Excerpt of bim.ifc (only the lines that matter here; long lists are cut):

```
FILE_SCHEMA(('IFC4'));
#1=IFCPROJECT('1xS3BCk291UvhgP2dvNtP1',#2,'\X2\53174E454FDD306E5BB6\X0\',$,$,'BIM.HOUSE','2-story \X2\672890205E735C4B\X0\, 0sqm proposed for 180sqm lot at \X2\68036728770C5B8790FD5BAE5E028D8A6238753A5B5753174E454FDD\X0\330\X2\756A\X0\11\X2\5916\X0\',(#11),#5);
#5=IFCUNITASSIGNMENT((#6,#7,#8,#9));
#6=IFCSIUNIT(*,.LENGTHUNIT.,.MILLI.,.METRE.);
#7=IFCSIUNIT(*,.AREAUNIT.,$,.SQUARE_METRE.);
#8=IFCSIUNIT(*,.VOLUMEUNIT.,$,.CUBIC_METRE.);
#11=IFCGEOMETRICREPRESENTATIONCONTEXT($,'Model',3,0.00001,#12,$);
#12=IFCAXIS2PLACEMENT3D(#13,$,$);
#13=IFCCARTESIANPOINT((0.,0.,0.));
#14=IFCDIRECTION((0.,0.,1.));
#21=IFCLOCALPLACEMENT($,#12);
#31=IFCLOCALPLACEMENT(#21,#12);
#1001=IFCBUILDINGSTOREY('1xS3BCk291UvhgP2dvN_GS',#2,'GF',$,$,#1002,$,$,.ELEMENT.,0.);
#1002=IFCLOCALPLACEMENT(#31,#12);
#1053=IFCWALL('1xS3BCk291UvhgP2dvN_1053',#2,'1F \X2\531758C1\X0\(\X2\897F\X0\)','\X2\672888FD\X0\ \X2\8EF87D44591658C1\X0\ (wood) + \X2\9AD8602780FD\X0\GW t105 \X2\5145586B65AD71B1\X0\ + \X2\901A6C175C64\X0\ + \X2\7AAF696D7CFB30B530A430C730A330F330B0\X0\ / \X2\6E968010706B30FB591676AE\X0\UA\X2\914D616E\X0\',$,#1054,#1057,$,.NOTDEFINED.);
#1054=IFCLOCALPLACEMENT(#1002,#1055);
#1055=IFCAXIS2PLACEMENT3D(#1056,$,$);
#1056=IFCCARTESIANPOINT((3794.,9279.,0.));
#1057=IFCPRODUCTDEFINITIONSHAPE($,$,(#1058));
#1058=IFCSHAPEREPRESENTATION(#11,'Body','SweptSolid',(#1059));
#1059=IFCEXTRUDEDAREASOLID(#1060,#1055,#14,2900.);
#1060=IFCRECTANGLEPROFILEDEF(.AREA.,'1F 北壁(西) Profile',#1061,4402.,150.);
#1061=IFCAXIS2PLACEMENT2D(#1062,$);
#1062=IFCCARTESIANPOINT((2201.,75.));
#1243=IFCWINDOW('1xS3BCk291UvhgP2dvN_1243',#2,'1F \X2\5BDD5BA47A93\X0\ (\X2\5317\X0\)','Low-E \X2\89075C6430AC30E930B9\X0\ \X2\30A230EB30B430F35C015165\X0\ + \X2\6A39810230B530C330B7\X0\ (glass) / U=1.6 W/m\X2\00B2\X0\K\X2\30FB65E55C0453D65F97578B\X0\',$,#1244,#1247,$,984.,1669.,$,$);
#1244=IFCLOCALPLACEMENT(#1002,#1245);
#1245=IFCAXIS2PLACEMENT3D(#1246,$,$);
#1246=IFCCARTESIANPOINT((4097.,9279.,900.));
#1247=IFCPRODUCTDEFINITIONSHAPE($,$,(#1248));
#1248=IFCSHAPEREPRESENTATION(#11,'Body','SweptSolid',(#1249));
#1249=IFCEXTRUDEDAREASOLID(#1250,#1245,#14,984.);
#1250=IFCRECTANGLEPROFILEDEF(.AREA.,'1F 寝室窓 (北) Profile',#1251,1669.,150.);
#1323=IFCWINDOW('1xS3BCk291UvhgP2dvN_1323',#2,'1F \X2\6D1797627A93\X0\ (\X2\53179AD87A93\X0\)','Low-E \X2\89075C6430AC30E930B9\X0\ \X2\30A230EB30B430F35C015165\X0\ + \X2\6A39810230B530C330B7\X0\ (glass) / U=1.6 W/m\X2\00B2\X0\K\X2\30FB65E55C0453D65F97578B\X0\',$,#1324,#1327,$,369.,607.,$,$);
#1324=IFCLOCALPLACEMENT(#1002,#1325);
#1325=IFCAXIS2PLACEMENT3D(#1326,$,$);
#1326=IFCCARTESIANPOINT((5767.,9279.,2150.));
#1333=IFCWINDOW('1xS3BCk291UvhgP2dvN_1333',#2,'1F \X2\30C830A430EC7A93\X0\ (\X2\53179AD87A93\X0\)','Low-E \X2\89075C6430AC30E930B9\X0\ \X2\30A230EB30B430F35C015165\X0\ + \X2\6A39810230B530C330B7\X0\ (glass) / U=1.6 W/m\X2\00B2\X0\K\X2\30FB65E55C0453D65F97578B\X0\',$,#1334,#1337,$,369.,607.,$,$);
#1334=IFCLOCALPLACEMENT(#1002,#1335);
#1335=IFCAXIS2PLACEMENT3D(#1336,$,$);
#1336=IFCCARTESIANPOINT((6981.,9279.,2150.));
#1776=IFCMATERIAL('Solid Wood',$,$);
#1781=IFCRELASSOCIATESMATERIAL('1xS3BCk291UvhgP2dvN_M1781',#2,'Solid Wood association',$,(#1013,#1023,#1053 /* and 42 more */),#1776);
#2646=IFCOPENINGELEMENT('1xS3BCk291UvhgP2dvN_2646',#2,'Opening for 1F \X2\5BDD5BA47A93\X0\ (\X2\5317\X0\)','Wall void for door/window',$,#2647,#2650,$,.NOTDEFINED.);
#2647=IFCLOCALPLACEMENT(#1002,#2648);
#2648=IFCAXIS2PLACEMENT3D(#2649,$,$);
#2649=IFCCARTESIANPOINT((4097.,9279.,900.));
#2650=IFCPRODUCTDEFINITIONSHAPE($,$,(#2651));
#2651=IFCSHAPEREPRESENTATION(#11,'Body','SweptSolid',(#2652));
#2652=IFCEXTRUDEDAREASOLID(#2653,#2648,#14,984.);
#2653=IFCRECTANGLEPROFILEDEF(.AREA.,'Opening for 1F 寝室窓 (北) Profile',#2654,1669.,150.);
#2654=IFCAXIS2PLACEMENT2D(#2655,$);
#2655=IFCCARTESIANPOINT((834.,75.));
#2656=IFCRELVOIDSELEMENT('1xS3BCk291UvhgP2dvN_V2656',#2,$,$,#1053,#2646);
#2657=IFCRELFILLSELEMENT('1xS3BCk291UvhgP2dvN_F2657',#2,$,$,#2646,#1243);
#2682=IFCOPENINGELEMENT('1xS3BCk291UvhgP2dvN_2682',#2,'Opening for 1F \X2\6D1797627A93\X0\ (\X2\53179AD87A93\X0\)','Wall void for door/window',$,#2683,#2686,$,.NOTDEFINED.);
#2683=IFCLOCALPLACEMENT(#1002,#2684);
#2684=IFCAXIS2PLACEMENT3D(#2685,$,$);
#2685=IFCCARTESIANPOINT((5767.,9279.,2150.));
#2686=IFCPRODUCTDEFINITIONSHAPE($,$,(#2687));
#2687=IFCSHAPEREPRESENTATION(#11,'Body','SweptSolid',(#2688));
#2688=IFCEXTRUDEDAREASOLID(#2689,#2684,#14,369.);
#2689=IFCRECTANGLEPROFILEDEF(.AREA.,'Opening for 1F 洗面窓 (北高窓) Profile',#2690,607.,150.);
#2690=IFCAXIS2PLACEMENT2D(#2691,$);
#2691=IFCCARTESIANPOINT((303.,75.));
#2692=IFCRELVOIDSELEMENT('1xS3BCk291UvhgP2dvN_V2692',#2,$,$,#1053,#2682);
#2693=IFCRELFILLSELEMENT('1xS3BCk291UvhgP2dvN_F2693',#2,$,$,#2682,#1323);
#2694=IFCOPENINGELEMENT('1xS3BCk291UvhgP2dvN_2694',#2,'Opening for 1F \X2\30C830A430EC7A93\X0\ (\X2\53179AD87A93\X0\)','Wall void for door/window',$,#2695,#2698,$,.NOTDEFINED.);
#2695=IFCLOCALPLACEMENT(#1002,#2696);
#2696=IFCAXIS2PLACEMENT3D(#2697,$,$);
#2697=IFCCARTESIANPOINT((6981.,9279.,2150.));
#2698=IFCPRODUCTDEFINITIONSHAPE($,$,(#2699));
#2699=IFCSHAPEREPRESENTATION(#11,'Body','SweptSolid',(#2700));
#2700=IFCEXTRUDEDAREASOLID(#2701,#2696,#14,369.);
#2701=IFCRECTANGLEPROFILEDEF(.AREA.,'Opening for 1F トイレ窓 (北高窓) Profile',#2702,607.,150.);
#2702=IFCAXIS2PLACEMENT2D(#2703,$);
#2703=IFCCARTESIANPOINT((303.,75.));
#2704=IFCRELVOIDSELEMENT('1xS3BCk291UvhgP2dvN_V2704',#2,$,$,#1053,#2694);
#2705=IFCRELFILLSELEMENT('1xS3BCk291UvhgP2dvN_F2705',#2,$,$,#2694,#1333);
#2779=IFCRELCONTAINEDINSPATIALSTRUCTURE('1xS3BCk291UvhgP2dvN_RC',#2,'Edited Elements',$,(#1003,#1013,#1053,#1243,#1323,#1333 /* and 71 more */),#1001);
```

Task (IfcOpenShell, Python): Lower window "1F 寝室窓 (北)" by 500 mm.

```python
import numpy as np
import ifcopenshell
import ifcopenshell.api.geometry
import ifcopenshell.util.placement
import ifcopenshell.util.unit

model = ifcopenshell.open("bim.ifc")
unit_scale = ifcopenshell.util.unit.calculate_unit_scale(model)

window = model.by_guid("1xS3BCk291UvhgP2dvN_1243")
opening = window.FillsVoids[0].RelatingOpeningElement
dz = -500.0

shift = np.array([0.0, 0.0, dz])
# The window is not placed relative to its opening, so move both.
for product in (opening, window):
    matrix = ifcopenshell.util.placement.get_local_placement(product.ObjectPlacement)
    matrix[:3, 3] += shift
    ifcopenshell.api.geometry.edit_object_placement(model, product=product, matrix=matrix, is_si=False)

print(f"moved by {dz * unit_scale:+.3f} m")

model.write("bim-out.ifc")
```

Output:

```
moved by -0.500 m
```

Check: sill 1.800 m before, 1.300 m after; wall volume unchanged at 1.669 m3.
